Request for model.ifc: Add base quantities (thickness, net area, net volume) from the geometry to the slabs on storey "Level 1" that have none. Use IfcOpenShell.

First a look at what the model holds.

```python
import ifcopenshell
import ifcopenshell.util.element
import ifcopenshell.util.unit

model = ifcopenshell.open("model.ifc")
print(model.schema)
for unit_type in ("LENGTHUNIT", "AREAUNIT", "VOLUMEUNIT"):
    print(unit_type, ifcopenshell.util.unit.calculate_unit_scale(model, unit_type))
storey = next(s for s in model.by_type("IfcBuildingStorey") if s.Name == "Level 1")
slabs = [e for e in ifcopenshell.util.element.get_decomposition(storey) if e.is_a("IfcSlab")]
for e in sorted(slabs, key=lambda e: e.id()):
    print(e.id(), e.is_a(), e.Name, list(ifcopenshell.util.element.get_psets(e, qtos_only=True)), sep=" | ")
```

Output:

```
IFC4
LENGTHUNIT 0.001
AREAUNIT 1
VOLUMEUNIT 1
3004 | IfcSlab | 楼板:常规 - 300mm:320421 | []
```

```python
import ifcopenshell
import ifcopenshell.api.pset
import ifcopenshell.geom
import ifcopenshell.util.element
import ifcopenshell.util.shape
import ifcopenshell.util.unit

model = ifcopenshell.open("model.ifc")
unit_scale = ifcopenshell.util.unit.calculate_unit_scale(model)
area_scale = ifcopenshell.util.unit.calculate_unit_scale(model, "AREAUNIT")
volume_scale = ifcopenshell.util.unit.calculate_unit_scale(model, "VOLUMEUNIT")
settings = ifcopenshell.geom.settings()

storey = next(s for s in model.by_type("IfcBuildingStorey") if s.Name == "Level 1")
slabs = [e for e in ifcopenshell.util.element.get_decomposition(storey) if e.is_a("IfcSlab")]

for e in sorted(slabs, key=lambda e: e.id()):
    if ifcopenshell.util.element.get_psets(e, qtos_only=True, should_inherit=False):
        continue
    # Geometry comes back in metres, in the element's own axes.
    shape = ifcopenshell.geom.create_shape(settings, e)
    values = {
        "Width": ifcopenshell.util.shape.get_z(shape.geometry) / unit_scale,
        "NetArea": ifcopenshell.util.shape.get_footprint_area(shape.geometry) / area_scale,
        "NetVolume": ifcopenshell.util.shape.get_volume(shape.geometry) / volume_scale,
    }
    qto = ifcopenshell.api.pset.add_qto(model, product=e, name="Qto_SlabBaseQuantities")
    ifcopenshell.api.pset.edit_qto(model, qto=qto, properties=values)
    print(e.id(), {k: round(v, 3) for k, v in values.items()})

model.write("model_updated.ifc")
```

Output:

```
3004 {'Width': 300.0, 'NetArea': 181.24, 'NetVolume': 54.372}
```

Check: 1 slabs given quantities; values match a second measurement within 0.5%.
